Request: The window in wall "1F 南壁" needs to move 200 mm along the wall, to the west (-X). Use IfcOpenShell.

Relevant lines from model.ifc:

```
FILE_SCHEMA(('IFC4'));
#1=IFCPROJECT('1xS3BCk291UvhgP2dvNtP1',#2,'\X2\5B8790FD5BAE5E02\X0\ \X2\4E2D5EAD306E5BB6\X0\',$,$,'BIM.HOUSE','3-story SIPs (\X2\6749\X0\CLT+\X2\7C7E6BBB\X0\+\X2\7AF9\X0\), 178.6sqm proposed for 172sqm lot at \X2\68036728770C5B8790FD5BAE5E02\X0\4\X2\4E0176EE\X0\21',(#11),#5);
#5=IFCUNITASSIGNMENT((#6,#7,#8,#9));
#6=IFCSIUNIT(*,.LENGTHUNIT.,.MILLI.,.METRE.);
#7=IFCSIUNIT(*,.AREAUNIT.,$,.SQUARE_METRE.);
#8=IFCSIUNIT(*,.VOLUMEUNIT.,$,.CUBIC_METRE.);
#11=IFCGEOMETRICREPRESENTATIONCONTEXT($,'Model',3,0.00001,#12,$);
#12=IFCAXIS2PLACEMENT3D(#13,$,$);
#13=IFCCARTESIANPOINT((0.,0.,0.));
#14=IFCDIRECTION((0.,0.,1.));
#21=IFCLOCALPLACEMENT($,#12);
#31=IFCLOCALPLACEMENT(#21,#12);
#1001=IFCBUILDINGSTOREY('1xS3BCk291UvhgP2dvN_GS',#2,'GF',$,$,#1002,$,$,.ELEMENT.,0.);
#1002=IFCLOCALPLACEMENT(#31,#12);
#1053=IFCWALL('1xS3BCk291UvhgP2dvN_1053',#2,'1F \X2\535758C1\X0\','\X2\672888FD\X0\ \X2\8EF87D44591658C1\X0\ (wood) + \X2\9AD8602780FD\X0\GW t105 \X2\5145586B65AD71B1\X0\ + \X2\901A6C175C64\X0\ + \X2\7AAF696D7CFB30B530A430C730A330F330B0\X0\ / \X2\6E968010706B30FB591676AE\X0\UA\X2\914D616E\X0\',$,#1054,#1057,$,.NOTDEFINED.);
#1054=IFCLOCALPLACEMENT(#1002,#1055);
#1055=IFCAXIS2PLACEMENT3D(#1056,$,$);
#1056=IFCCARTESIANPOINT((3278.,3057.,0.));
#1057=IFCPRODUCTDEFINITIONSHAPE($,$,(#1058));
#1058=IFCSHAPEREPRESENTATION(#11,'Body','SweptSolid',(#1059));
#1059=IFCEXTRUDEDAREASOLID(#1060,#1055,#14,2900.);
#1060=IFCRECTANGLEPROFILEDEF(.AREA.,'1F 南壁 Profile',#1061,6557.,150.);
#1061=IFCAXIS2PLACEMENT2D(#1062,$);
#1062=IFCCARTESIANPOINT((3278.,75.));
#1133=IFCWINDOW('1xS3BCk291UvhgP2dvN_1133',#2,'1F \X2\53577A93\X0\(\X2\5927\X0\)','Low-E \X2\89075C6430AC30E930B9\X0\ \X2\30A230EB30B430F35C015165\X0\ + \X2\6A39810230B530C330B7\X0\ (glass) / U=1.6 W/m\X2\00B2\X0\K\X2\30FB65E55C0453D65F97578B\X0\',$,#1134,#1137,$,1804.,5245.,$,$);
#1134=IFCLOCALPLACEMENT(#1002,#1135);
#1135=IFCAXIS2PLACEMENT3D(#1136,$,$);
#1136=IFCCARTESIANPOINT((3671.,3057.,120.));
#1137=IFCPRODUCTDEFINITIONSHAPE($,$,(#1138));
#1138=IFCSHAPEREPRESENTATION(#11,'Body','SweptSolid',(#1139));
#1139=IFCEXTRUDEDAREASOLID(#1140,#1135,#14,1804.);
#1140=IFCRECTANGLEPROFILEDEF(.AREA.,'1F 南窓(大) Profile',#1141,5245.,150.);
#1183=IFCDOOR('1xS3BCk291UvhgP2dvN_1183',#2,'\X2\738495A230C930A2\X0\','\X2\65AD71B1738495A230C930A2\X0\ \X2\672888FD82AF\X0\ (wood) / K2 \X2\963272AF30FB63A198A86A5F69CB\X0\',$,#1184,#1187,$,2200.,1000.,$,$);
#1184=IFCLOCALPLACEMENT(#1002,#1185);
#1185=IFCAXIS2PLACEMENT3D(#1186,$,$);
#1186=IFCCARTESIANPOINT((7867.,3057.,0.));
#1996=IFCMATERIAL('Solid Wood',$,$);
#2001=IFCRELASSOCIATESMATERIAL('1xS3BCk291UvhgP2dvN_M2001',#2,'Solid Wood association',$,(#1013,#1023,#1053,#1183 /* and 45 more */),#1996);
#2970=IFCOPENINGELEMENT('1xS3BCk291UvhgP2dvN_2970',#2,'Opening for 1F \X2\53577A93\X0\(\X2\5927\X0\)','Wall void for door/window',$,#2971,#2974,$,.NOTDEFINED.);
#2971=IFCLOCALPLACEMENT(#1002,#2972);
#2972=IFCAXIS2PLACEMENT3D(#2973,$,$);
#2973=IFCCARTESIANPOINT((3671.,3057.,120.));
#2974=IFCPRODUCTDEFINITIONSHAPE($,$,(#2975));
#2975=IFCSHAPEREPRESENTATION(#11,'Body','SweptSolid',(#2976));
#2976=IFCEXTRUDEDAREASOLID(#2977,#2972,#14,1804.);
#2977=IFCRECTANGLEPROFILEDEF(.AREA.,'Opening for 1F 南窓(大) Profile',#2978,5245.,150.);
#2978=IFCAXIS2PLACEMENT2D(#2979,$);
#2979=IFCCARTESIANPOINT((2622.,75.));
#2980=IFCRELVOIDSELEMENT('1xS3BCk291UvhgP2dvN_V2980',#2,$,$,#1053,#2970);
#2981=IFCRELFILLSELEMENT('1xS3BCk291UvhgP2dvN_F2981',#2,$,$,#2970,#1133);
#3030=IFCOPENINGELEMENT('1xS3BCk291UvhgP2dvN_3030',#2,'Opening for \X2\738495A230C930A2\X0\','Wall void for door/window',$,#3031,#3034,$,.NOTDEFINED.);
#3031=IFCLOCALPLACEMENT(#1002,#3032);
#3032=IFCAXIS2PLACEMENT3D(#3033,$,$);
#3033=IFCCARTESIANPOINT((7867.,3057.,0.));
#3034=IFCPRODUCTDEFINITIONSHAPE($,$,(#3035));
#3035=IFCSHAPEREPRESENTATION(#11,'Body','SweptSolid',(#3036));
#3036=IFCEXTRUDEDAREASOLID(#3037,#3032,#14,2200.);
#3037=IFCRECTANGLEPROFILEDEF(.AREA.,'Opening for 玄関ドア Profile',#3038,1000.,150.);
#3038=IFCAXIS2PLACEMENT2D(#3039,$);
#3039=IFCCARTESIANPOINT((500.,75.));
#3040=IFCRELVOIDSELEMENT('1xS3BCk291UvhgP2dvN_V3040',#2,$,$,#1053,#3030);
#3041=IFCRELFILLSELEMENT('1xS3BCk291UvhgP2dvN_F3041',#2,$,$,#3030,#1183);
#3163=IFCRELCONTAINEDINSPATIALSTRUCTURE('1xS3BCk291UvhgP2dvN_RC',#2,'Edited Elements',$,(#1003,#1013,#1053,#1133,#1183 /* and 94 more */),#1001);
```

```python
import ifcopenshell
import ifcopenshell.api.geometry
import ifcopenshell.util.placement

model = ifcopenshell.open("model.ifc")

window = model.by_guid("1xS3BCk291UvhgP2dvN_1133")
opening = window.FillsVoids[0].RelatingOpeningElement
wall = opening.VoidsElements[0].RelatingBuildingElement

wall_matrix = ifcopenshell.util.placement.get_local_placement(wall.ObjectPlacement)
shift = wall_matrix[:3, 0] * -200.0
before = ifcopenshell.util.placement.get_local_placement(window.ObjectPlacement)[:3, 3].copy()

# The window is not placed relative to its opening, so move both.
for product in (opening, window):
    matrix = ifcopenshell.util.placement.get_local_placement(product.ObjectPlacement)
    matrix[:3, 3] += shift
    ifcopenshell.api.geometry.edit_object_placement(model, product=product, matrix=matrix, is_si=False)

after = ifcopenshell.util.placement.get_local_placement(window.ObjectPlacement)[:3, 3]
print("window moved by", (after - before).round(3) + 0.0)

model.write("model_v2.ifc")
```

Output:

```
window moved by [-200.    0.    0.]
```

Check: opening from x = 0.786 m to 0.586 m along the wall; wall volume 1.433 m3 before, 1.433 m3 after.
